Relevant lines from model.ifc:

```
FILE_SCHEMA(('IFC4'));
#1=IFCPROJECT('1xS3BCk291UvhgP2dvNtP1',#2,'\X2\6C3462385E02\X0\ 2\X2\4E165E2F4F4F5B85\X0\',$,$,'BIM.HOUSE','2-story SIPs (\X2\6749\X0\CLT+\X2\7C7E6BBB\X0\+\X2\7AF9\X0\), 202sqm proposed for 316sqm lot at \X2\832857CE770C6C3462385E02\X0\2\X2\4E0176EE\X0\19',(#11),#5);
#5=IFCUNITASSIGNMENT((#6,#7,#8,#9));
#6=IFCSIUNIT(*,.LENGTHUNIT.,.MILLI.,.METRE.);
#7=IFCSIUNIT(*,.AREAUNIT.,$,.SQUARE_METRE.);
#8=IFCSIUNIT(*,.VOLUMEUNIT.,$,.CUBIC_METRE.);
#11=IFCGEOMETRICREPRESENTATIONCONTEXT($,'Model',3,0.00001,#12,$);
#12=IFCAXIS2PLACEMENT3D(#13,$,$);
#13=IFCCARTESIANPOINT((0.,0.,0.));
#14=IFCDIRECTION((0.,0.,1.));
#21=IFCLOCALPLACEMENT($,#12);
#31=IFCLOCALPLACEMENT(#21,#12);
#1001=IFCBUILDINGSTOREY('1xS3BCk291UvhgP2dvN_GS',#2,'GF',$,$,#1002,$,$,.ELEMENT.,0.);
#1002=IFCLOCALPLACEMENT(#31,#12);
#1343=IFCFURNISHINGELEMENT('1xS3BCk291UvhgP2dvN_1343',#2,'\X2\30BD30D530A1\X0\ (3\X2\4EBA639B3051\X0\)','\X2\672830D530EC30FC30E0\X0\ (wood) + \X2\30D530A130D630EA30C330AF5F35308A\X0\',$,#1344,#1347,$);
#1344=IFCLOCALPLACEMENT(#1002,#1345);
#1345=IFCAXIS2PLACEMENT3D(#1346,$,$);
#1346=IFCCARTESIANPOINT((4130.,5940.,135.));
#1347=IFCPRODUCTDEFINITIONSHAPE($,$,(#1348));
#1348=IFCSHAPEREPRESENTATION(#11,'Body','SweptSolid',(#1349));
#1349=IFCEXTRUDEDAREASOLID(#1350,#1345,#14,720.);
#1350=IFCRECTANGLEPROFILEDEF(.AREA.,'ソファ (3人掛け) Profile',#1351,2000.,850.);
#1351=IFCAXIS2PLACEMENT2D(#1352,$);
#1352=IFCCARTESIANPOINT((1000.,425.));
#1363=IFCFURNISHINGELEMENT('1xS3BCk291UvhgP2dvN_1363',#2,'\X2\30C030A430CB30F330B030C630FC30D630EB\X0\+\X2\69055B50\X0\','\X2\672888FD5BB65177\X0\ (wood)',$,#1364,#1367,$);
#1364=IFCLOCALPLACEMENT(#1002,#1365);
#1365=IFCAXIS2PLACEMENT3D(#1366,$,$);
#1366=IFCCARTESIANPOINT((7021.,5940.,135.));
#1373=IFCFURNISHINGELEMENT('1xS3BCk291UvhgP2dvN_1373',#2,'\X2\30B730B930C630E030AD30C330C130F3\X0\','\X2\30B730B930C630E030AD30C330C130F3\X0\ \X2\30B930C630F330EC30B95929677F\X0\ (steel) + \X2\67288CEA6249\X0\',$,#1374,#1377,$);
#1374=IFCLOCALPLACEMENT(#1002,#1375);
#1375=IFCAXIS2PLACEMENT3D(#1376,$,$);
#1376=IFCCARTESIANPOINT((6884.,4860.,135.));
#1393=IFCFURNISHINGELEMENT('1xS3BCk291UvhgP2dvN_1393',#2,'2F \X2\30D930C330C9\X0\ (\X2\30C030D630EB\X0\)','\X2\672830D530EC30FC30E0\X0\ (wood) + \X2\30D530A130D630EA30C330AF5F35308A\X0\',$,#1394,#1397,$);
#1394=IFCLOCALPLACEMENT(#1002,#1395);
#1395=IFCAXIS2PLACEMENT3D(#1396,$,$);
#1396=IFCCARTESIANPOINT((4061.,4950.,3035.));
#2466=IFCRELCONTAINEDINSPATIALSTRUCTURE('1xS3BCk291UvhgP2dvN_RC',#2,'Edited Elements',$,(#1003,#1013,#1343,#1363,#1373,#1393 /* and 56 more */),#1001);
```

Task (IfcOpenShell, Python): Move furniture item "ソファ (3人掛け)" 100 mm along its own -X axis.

```python
import ifcopenshell
import ifcopenshell.api.geometry
import ifcopenshell.util.placement
import ifcopenshell.util.unit

model = ifcopenshell.open("model.ifc")
unit_scale = ifcopenshell.util.unit.calculate_unit_scale(model)

item = model.by_guid("1xS3BCk291UvhgP2dvN_1343")
matrix = ifcopenshell.util.placement.get_local_placement(item.ObjectPlacement)
matrix[:3, 3] -= matrix[:3, 0] * 0.1 / unit_scale
ifcopenshell.api.geometry.edit_object_placement(model, product=item, matrix=matrix, is_si=False)

print(ifcopenshell.util.placement.get_local_placement(item.ObjectPlacement).round(3) + 0.0)

model.write("model_v2.ifc")
```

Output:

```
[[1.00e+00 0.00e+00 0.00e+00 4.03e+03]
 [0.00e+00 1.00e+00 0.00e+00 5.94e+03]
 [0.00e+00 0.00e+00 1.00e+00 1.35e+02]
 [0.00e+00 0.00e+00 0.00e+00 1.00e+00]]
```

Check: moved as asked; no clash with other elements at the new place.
